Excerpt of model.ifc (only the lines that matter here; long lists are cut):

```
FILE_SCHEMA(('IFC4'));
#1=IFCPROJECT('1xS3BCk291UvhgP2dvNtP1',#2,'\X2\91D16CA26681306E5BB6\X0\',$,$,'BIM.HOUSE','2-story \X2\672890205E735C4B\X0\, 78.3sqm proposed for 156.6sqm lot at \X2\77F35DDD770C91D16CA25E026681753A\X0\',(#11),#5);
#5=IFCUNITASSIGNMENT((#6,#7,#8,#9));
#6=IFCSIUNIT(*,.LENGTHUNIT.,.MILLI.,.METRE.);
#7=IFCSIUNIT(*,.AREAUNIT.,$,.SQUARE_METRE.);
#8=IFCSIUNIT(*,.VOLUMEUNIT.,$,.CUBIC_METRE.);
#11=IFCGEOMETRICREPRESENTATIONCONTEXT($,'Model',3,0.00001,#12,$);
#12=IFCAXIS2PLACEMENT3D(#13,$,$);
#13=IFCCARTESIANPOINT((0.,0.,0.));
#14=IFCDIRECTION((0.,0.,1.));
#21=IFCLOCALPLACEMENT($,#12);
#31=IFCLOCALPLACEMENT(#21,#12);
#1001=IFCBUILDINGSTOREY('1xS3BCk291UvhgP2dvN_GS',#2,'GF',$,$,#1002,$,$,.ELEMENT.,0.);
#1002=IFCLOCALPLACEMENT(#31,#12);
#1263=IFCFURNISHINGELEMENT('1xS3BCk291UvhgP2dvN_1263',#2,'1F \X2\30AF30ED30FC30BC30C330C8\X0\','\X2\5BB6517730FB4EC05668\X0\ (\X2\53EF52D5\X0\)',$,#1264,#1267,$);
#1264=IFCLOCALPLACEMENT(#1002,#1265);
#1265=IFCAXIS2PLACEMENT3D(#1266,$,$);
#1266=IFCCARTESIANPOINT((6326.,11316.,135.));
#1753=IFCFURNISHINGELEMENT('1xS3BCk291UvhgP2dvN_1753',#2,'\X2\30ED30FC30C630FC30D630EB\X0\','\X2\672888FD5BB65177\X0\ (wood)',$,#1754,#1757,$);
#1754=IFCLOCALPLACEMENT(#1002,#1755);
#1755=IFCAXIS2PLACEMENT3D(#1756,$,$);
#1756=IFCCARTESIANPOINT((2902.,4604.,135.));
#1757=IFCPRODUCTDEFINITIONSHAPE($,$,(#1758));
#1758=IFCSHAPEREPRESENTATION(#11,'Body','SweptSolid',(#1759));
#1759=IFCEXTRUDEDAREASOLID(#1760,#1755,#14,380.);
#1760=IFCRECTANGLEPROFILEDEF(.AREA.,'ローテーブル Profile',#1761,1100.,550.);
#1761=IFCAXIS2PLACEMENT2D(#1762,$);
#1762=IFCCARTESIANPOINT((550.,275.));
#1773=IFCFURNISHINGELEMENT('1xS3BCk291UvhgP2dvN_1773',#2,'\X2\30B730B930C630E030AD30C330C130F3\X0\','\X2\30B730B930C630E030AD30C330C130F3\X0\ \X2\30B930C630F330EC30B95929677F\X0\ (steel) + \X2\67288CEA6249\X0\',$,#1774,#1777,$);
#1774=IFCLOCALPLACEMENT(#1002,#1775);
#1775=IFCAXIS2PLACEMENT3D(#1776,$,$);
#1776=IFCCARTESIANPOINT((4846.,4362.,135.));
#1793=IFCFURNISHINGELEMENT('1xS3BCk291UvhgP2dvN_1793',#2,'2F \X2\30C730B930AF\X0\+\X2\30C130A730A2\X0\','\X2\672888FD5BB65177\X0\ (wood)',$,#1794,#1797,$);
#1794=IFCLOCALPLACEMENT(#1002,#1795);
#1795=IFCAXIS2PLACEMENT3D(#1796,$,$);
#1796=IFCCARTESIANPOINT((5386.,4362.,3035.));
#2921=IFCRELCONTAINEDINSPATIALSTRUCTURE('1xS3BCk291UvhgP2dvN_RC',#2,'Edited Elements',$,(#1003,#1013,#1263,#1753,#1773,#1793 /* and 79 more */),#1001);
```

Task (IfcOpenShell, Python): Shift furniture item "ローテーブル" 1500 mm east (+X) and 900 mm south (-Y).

```python
import ifcopenshell
import ifcopenshell.api.geometry
import ifcopenshell.util.placement

model = ifcopenshell.open("model.ifc")

item = model.by_guid("1xS3BCk291UvhgP2dvN_1753")
matrix = ifcopenshell.util.placement.get_local_placement(item.ObjectPlacement)
matrix[0, 3] += 1500.0
matrix[1, 3] -= 900.0
ifcopenshell.api.geometry.edit_object_placement(model, product=item, matrix=matrix, is_si=False)

print(ifcopenshell.util.placement.get_local_placement(item.ObjectPlacement).round(3) + 0.0)

model.write("model-out.ifc")
```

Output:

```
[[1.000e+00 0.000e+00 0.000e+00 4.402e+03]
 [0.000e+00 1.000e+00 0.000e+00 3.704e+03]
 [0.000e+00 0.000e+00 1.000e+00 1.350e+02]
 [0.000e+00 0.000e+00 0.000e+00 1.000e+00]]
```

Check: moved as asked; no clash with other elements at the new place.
